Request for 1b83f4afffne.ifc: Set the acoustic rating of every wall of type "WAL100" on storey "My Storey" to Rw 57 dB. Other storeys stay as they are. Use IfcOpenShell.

First a look at what the model holds.

```python
import ifcopenshell
import ifcopenshell.util.element

model = ifcopenshell.open("1b83f4afffne.ifc")
print(model.schema)
storey = next(s for s in model.by_type("IfcBuildingStorey") if s.Name == "My Storey")
walls = [e for e in ifcopenshell.util.element.get_decomposition(storey) if e.is_a("IfcWall")]
seen = {}
for e in walls:
    element_type = ifcopenshell.util.element.get_type(e)
    key = (element_type.Name if element_type != e and element_type else None, ifcopenshell.util.element.get_pset(e, "Pset_WallCommon", "AcousticRating"))
    seen[key] = seen.get(key, 0) + 1
for (name, value), count in sorted(seen.items(), key=str):
    print(count, "x", name, "|", value)
```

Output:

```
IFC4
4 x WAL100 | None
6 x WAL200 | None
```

```python
import ifcopenshell
import ifcopenshell.api.pset
import ifcopenshell.util.element

model = ifcopenshell.open("1b83f4afffne.ifc")

storey = next(s for s in model.by_type("IfcBuildingStorey") if s.Name == "My Storey")
walls = [e for e in ifcopenshell.util.element.get_decomposition(storey) if e.is_a("IfcWall")]

count = 0
for e in walls:
    element_type = ifcopenshell.util.element.get_type(e)
    if element_type in (None, e) or element_type.Name != "WAL100":
        continue
    # add_pset returns the element's existing set when there is one.
    pset = ifcopenshell.api.pset.add_pset(model, product=e, name="Pset_WallCommon")
    ifcopenshell.api.pset.edit_pset(model, pset=pset, properties={"AcousticRating": "Rw 57 dB"})
    count += 1

print(count, "walls updated")

model.write("1b83f4afffne_edited.ifc")
```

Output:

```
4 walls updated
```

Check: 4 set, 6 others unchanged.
